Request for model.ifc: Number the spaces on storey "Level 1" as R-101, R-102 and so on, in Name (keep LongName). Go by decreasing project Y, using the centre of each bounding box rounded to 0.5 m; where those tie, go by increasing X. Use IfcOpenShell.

First a look at what the model holds.

```python
import ifcopenshell
import ifcopenshell.util.element
import ifcopenshell.util.placement

model = ifcopenshell.open("model.ifc")
print(model.schema)
storey = next(s for s in model.by_type("IfcBuildingStorey") if s.Name == "Level 1")
spaces = [e for e in ifcopenshell.util.element.get_decomposition(storey) if e.is_a("IfcSpace")]
for e in sorted(spaces, key=lambda e: e.id()):
    origin = ifcopenshell.util.placement.get_local_placement(e.ObjectPlacement)[:3, 3]
    print(e.id(), e.Name, e.LongName, origin.round(2) + 0.0, sep=" | ")
```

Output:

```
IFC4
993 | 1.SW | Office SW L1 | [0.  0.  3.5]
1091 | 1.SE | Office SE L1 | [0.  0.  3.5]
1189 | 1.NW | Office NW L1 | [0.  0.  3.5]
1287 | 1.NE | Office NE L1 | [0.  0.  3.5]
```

```python
import ifcopenshell
import ifcopenshell.geom
import ifcopenshell.util.element
import ifcopenshell.util.shape

model = ifcopenshell.open("model.ifc")
settings = ifcopenshell.geom.settings()
settings.set("use-world-coords", True)


def centre(element):
    shape = ifcopenshell.geom.create_shape(settings, element)
    return ifcopenshell.util.shape.get_bbox_centroid(shape.geometry)


storey = next(s for s in model.by_type("IfcBuildingStorey") if s.Name == "Level 1")
spaces = [e for e in ifcopenshell.util.element.get_decomposition(storey) if e.is_a("IfcSpace")]

# Insertion points can sit at a corner or the storey origin, so sort by the geometry (in metres).
centres = {e: centre(e) for e in spaces}
spaces.sort(key=lambda e: (-round(centres[e][1] / 0.5), centres[e][0]))

for i, e in enumerate(spaces, start=1):
    number = f"R-1{i:02d}"
    e.Name = number
    print(e.id(), number)

model.write("model-out.ifc")
```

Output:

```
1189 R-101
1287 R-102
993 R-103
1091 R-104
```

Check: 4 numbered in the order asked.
